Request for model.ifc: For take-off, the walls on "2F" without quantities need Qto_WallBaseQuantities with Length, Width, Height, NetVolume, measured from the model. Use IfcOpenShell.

First a look at what the model holds.

```python
import ifcopenshell
import ifcopenshell.util.element
import ifcopenshell.util.unit

model = ifcopenshell.open("model.ifc")
print(model.schema)
for unit_type in ("LENGTHUNIT", "AREAUNIT", "VOLUMEUNIT"):
    print(unit_type, ifcopenshell.util.unit.calculate_unit_scale(model, unit_type))
storey = next(s for s in model.by_type("IfcBuildingStorey") if s.Name == "2F")
walls = [e for e in ifcopenshell.util.element.get_decomposition(storey) if e.is_a("IfcWall")]
for e in sorted(walls, key=lambda e: e.id()):
    print(e.id(), e.is_a(), e.Name, list(ifcopenshell.util.element.get_psets(e, qtos_only=True)), sep=" | ")
```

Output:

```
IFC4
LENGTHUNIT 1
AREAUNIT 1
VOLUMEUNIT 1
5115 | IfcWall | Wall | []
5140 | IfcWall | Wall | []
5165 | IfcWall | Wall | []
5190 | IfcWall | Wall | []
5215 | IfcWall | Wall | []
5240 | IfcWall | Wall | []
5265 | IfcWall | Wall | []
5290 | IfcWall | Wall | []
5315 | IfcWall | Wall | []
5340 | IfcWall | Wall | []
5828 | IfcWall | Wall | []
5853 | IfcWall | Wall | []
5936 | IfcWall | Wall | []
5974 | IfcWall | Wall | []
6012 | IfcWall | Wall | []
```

```python
import ifcopenshell
import ifcopenshell.api.pset
import ifcopenshell.geom
import ifcopenshell.util.element
import ifcopenshell.util.shape
import ifcopenshell.util.unit

model = ifcopenshell.open("model.ifc")
unit_scale = ifcopenshell.util.unit.calculate_unit_scale(model)
volume_scale = ifcopenshell.util.unit.calculate_unit_scale(model, "VOLUMEUNIT")
settings = ifcopenshell.geom.settings()

storey = next(s for s in model.by_type("IfcBuildingStorey") if s.Name == "2F")
walls = [e for e in ifcopenshell.util.element.get_decomposition(storey) if e.is_a("IfcWall")]

for e in sorted(walls, key=lambda e: e.id()):
    if ifcopenshell.util.element.get_psets(e, qtos_only=True, should_inherit=False):
        continue
    # Geometry comes back in metres, in the element's own axes.
    shape = ifcopenshell.geom.create_shape(settings, e)
    values = {
        "Length": ifcopenshell.util.shape.get_x(shape.geometry) / unit_scale,
        "Width": ifcopenshell.util.shape.get_y(shape.geometry) / unit_scale,
        "Height": ifcopenshell.util.shape.get_z(shape.geometry) / unit_scale,
        "NetVolume": ifcopenshell.util.shape.get_volume(shape.geometry) / volume_scale,
    }
    qto = ifcopenshell.api.pset.add_qto(model, product=e, name="Qto_WallBaseQuantities")
    ifcopenshell.api.pset.edit_qto(model, qto=qto, properties=values)
    print(e.id(), {k: round(v, 3) for k, v in values.items()})

model.write("model-out.ifc")
```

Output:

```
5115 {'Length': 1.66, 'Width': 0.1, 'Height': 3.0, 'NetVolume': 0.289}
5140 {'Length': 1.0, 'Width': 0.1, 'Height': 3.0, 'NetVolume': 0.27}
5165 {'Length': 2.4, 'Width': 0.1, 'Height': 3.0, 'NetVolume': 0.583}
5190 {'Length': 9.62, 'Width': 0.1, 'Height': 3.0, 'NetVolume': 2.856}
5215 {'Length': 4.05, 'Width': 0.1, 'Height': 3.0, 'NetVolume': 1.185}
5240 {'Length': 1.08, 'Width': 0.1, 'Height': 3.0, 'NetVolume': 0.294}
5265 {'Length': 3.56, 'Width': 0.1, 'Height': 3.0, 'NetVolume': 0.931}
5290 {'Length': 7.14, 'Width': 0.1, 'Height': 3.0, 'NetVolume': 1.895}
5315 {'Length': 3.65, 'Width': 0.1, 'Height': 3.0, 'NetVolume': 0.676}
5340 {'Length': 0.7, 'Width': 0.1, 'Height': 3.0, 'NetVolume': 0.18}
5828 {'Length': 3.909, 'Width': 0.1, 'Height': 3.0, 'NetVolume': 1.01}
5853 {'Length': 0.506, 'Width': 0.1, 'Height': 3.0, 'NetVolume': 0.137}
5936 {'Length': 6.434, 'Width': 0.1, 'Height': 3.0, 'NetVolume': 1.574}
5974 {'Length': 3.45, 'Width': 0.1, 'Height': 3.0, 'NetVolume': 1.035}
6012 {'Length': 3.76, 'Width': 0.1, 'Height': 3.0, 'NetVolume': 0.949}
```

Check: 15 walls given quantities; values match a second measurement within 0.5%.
